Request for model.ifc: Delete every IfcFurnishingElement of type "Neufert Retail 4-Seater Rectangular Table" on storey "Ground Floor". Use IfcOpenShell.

First a look at what the model holds.

```python
import ifcopenshell
import ifcopenshell.util.element

model = ifcopenshell.open("model.ifc")
print(model.schema)
storey = next(s for s in model.by_type("IfcBuildingStorey") if s.Name == "Ground Floor")
furniture = [e for e in ifcopenshell.util.element.get_decomposition(storey) if e.is_a("IfcFurnishingElement")]
seen = {}
for e in furniture:
    element_type = ifcopenshell.util.element.get_type(e)
    name = element_type.Name if element_type not in (None, e) else None
    seen[name] = seen.get(name, 0) + 1
for name, count in sorted(seen.items(), key=str):
    print(count, "x", name)
```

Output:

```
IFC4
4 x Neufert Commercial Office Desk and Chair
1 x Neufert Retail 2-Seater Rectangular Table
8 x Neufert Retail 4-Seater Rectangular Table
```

```python
import ifcopenshell
import ifcopenshell.api.root
import ifcopenshell.util.element

model = ifcopenshell.open("model.ifc")

storey = next(s for s in model.by_type("IfcBuildingStorey") if s.Name == "Ground Floor")
furniture = [e for e in ifcopenshell.util.element.get_decomposition(storey) if e.is_a("IfcFurnishingElement")]
targets = [e for e in furniture if (t := ifcopenshell.util.element.get_type(e)) not in (None, e) and t.Name == "Neufert Retail 4-Seater Rectangular Table"]

for e in targets:
    ifcopenshell.api.root.remove_product(model, product=e)
print(len(targets), "removed")

model.write("model_rev.ifc")
```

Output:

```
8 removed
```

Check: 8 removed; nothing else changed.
